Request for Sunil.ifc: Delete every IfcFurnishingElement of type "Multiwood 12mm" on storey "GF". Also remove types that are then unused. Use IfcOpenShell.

First a look at what the model holds.

```python
import ifcopenshell
import ifcopenshell.util.element

model = ifcopenshell.open("Sunil.ifc")
print(model.schema)
storey = next(s for s in model.by_type("IfcBuildingStorey") if s.Name == "GF")
furniture = [e for e in ifcopenshell.util.element.get_decomposition(storey) if e.is_a("IfcFurnishingElement")]
seen = {}
for e in furniture:
    element_type = ifcopenshell.util.element.get_type(e)
    name = element_type.Name if element_type not in (None, e) else None
    seen[name] = seen.get(name, 0) + 1
for name, count in sorted(seen.items(), key=str):
    print(count, "x", name)
```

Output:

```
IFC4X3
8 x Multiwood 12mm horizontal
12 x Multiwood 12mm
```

```python
import ifcopenshell
import ifcopenshell.api.root
import ifcopenshell.util.element

model = ifcopenshell.open("Sunil.ifc")

storey = next(s for s in model.by_type("IfcBuildingStorey") if s.Name == "GF")
furniture = [e for e in ifcopenshell.util.element.get_decomposition(storey) if e.is_a("IfcFurnishingElement")]
targets = [e for e in furniture if (t := ifcopenshell.util.element.get_type(e)) not in (None, e) and t.Name == "Multiwood 12mm"]
types = {ifcopenshell.util.element.get_type(e) for e in targets} - {None, *targets}

for e in targets:
    ifcopenshell.api.root.remove_product(model, product=e)
print(len(targets), "removed")

unused = [t for t in types if not ifcopenshell.util.element.get_types(t)]
for t in unused:
    ifcopenshell.api.root.remove_product(model, product=t)
print(len(unused), "unused types removed")

model.write("Sunil_updated.ifc")
```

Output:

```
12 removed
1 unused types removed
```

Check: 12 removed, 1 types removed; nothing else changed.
